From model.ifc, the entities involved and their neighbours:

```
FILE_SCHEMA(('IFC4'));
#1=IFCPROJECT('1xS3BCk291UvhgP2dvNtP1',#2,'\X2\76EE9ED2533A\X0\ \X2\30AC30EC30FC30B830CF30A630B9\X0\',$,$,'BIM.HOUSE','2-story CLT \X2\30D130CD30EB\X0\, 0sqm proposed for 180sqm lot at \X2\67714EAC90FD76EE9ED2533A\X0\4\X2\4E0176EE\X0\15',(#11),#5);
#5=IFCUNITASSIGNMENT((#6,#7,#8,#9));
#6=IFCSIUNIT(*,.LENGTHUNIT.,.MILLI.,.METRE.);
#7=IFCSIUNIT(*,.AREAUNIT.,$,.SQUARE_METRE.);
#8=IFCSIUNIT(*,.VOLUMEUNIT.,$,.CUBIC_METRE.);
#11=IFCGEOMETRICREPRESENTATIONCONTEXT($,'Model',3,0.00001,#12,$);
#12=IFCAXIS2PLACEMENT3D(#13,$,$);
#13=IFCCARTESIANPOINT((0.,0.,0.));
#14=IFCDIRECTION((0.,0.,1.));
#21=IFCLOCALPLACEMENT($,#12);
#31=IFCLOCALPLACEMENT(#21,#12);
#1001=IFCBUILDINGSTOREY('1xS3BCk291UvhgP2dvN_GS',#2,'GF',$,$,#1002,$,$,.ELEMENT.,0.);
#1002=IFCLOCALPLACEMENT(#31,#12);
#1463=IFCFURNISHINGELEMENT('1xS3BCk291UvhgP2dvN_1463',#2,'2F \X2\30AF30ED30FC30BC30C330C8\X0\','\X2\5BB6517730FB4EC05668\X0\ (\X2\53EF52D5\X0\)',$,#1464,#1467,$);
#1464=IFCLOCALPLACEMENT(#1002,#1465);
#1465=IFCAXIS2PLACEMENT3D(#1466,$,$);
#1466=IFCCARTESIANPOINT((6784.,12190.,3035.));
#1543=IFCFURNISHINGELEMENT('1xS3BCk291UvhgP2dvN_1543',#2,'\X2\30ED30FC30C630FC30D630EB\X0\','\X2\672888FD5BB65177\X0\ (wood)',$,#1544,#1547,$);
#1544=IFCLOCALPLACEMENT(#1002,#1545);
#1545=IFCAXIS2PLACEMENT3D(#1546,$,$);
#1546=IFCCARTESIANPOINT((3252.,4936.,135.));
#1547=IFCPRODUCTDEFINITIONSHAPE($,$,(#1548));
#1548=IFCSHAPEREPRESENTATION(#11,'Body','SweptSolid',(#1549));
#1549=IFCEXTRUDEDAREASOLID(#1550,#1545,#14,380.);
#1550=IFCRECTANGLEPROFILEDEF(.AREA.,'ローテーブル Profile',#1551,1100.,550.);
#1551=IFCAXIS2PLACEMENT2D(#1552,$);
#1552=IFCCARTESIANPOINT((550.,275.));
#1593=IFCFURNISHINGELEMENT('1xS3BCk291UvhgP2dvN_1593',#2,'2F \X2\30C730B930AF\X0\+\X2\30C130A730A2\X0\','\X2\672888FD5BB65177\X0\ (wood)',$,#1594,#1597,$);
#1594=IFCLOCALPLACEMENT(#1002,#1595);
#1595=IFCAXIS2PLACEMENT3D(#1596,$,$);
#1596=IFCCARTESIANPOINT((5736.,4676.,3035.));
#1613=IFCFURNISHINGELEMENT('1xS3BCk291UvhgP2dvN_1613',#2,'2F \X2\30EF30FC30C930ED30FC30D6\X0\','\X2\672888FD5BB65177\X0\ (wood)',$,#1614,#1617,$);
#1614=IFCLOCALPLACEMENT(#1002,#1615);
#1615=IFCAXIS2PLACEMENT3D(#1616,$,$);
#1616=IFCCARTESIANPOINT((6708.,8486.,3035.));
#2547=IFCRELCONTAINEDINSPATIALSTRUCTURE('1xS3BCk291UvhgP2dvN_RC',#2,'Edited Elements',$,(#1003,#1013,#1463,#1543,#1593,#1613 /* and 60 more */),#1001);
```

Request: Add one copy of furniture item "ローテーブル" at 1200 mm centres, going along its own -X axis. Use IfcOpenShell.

```python
import ifcopenshell
import ifcopenshell.api.geometry
import ifcopenshell.api.root
import ifcopenshell.util.element
import ifcopenshell.util.placement
import ifcopenshell.util.unit

model = ifcopenshell.open("model.ifc")
unit_scale = ifcopenshell.util.unit.calculate_unit_scale(model)


def reuse_history(source, copy):
    """copy_class also copies each property set's owner history, people and application; keep the originals."""
    for rel in copy.IsDefinedBy:
        if rel.is_a("IfcRelDefinesByProperties") and (history := rel.RelatingPropertyDefinition.OwnerHistory):
            rel.RelatingPropertyDefinition.OwnerHistory = source.OwnerHistory
            ifcopenshell.util.element.remove_deep2(model, history)


source = model.by_guid("1xS3BCk291UvhgP2dvN_1543")
base = ifcopenshell.util.placement.get_local_placement(source.ObjectPlacement)
step = -base[:3, 0] * 1.2 / unit_scale

for i in range(1, 2):
    copy = ifcopenshell.api.root.copy_class(model, product=source)
    copy.Representation = ifcopenshell.util.element.copy_deep(
        model, source.Representation, exclude=["IfcGeometricRepresentationContext", "IfcRepresentationMap"]
    )
    reuse_history(source, copy)
    matrix = base.copy()
    matrix[:3, 3] += i * step
    print("added at", matrix[:3, 3].round(3) + 0.0)
    ifcopenshell.api.geometry.edit_object_placement(model, product=copy, matrix=matrix, is_si=False)

model.write("model-out.ifc")
```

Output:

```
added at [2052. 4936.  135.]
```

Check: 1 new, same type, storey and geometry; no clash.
